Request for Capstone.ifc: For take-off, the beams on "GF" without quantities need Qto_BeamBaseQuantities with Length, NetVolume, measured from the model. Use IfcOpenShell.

First a look at what the model holds.

```python
import ifcopenshell
import ifcopenshell.util.element
import ifcopenshell.util.unit

model = ifcopenshell.open("Capstone.ifc")
print(model.schema)
for unit_type in ("LENGTHUNIT", "AREAUNIT", "VOLUMEUNIT"):
    print(unit_type, ifcopenshell.util.unit.calculate_unit_scale(model, unit_type))
storey = next(s for s in model.by_type("IfcBuildingStorey") if s.Name == "GF")
beams = [e for e in ifcopenshell.util.element.get_decomposition(storey) if e.is_a("IfcBeam")]
for e in sorted(beams, key=lambda e: e.id()):
    print(e.id(), e.is_a(), e.Name, list(ifcopenshell.util.element.get_psets(e, qtos_only=True)), sep=" | ")
```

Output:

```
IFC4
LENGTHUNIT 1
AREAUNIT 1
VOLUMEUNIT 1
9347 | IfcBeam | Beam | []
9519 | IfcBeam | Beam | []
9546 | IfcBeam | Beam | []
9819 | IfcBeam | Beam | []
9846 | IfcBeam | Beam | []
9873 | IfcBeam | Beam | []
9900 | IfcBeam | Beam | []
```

```python
import ifcopenshell
import ifcopenshell.api.pset
import ifcopenshell.geom
import ifcopenshell.util.element
import ifcopenshell.util.shape
import ifcopenshell.util.unit

model = ifcopenshell.open("Capstone.ifc")
unit_scale = ifcopenshell.util.unit.calculate_unit_scale(model)
volume_scale = ifcopenshell.util.unit.calculate_unit_scale(model, "VOLUMEUNIT")
settings = ifcopenshell.geom.settings()

storey = next(s for s in model.by_type("IfcBuildingStorey") if s.Name == "GF")
beams = [e for e in ifcopenshell.util.element.get_decomposition(storey) if e.is_a("IfcBeam")]

for e in sorted(beams, key=lambda e: e.id()):
    if ifcopenshell.util.element.get_psets(e, qtos_only=True, should_inherit=False):
        continue
    # Geometry comes back in metres, in the element's own axes.
    shape = ifcopenshell.geom.create_shape(settings, e)
    values = {
        "Length": ifcopenshell.util.shape.get_max_xyz(shape.geometry) / unit_scale,
        "NetVolume": ifcopenshell.util.shape.get_volume(shape.geometry) / volume_scale,
    }
    qto = ifcopenshell.api.pset.add_qto(model, product=e, name="Qto_BeamBaseQuantities")
    ifcopenshell.api.pset.edit_qto(model, qto=qto, properties=values)
    print(e.id(), {k: round(v, 3) for k, v in values.items()})

model.write("Capstone_updated.ifc")
```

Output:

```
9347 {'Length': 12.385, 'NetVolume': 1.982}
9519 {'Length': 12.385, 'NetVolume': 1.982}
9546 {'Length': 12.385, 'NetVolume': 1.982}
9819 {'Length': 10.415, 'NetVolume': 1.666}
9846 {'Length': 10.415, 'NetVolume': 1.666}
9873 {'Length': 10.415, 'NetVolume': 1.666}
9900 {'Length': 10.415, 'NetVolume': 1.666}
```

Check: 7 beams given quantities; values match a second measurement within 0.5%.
